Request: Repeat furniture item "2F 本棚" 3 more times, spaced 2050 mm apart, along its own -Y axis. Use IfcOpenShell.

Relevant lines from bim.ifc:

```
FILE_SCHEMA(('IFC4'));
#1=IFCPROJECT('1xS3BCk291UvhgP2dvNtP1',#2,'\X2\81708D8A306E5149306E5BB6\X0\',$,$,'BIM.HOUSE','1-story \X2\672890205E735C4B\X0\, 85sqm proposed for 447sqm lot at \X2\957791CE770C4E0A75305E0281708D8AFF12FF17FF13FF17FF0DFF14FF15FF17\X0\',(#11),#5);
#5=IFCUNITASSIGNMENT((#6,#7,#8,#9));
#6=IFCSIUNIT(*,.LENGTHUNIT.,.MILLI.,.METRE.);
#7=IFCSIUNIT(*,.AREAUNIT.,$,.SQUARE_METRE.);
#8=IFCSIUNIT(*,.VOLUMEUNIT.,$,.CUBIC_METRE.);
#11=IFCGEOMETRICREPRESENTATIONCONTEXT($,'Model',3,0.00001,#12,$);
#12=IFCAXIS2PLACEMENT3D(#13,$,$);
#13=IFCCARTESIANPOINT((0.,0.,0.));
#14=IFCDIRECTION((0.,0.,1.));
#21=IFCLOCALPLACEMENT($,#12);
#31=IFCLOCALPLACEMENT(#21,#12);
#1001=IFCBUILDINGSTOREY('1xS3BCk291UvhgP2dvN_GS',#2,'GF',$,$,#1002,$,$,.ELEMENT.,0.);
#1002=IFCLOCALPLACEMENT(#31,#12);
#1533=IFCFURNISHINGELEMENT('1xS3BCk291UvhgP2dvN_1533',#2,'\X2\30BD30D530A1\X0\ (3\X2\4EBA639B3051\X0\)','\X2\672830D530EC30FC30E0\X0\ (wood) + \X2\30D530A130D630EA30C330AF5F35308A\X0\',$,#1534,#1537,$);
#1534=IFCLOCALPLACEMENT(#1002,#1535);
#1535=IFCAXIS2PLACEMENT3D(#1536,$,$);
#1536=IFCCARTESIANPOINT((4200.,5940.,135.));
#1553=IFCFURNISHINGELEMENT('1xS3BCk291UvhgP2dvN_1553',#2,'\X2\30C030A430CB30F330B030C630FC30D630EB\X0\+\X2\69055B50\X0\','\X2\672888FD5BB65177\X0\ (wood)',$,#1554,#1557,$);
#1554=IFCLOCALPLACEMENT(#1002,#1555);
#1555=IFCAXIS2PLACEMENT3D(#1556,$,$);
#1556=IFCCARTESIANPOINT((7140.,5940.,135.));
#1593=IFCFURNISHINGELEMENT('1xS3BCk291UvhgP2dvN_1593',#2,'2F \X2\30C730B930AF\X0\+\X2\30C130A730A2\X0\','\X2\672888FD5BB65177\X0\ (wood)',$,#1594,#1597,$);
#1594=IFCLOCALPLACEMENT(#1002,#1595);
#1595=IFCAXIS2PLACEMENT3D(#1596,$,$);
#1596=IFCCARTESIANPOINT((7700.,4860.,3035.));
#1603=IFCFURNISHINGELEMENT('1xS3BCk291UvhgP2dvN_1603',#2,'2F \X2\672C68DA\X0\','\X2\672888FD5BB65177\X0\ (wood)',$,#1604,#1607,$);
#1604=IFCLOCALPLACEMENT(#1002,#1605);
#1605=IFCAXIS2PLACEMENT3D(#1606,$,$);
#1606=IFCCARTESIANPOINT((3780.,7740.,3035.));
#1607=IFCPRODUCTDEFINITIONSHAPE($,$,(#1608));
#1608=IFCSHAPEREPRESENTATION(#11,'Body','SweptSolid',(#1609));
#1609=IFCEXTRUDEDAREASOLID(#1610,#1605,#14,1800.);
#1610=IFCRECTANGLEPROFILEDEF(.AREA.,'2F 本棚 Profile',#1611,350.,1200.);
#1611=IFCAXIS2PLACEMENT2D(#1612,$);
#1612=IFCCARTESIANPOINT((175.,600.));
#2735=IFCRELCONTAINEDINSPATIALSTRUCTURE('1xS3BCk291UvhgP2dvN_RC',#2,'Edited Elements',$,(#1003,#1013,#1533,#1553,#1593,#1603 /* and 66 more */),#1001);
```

```python
import ifcopenshell
import ifcopenshell.api.geometry
import ifcopenshell.api.root
import ifcopenshell.util.element
import ifcopenshell.util.placement

model = ifcopenshell.open("bim.ifc")


def reuse_history(source, copy):
    """copy_class also copies each property set's owner history, people and application; keep the originals."""
    for rel in copy.IsDefinedBy:
        if rel.is_a("IfcRelDefinesByProperties") and (history := rel.RelatingPropertyDefinition.OwnerHistory):
            rel.RelatingPropertyDefinition.OwnerHistory = source.OwnerHistory
            ifcopenshell.util.element.remove_deep2(model, history)


source = model.by_id(1603)
base = ifcopenshell.util.placement.get_local_placement(source.ObjectPlacement)
step = -base[:3, 1] * 2050.0

for i in range(1, 4):
    copy = ifcopenshell.api.root.copy_class(model, product=source)
    copy.Representation = ifcopenshell.util.element.copy_deep(
        model, source.Representation, exclude=["IfcGeometricRepresentationContext", "IfcRepresentationMap"]
    )
    reuse_history(source, copy)
    matrix = base.copy()
    matrix[:3, 3] += i * step
    print("added at", matrix[:3, 3].round(3) + 0.0)
    ifcopenshell.api.geometry.edit_object_placement(model, product=copy, matrix=matrix, is_si=False)

model.write("bim_v2.ifc")
```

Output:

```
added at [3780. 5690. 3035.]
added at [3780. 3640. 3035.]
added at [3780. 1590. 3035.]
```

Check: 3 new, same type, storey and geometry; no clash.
